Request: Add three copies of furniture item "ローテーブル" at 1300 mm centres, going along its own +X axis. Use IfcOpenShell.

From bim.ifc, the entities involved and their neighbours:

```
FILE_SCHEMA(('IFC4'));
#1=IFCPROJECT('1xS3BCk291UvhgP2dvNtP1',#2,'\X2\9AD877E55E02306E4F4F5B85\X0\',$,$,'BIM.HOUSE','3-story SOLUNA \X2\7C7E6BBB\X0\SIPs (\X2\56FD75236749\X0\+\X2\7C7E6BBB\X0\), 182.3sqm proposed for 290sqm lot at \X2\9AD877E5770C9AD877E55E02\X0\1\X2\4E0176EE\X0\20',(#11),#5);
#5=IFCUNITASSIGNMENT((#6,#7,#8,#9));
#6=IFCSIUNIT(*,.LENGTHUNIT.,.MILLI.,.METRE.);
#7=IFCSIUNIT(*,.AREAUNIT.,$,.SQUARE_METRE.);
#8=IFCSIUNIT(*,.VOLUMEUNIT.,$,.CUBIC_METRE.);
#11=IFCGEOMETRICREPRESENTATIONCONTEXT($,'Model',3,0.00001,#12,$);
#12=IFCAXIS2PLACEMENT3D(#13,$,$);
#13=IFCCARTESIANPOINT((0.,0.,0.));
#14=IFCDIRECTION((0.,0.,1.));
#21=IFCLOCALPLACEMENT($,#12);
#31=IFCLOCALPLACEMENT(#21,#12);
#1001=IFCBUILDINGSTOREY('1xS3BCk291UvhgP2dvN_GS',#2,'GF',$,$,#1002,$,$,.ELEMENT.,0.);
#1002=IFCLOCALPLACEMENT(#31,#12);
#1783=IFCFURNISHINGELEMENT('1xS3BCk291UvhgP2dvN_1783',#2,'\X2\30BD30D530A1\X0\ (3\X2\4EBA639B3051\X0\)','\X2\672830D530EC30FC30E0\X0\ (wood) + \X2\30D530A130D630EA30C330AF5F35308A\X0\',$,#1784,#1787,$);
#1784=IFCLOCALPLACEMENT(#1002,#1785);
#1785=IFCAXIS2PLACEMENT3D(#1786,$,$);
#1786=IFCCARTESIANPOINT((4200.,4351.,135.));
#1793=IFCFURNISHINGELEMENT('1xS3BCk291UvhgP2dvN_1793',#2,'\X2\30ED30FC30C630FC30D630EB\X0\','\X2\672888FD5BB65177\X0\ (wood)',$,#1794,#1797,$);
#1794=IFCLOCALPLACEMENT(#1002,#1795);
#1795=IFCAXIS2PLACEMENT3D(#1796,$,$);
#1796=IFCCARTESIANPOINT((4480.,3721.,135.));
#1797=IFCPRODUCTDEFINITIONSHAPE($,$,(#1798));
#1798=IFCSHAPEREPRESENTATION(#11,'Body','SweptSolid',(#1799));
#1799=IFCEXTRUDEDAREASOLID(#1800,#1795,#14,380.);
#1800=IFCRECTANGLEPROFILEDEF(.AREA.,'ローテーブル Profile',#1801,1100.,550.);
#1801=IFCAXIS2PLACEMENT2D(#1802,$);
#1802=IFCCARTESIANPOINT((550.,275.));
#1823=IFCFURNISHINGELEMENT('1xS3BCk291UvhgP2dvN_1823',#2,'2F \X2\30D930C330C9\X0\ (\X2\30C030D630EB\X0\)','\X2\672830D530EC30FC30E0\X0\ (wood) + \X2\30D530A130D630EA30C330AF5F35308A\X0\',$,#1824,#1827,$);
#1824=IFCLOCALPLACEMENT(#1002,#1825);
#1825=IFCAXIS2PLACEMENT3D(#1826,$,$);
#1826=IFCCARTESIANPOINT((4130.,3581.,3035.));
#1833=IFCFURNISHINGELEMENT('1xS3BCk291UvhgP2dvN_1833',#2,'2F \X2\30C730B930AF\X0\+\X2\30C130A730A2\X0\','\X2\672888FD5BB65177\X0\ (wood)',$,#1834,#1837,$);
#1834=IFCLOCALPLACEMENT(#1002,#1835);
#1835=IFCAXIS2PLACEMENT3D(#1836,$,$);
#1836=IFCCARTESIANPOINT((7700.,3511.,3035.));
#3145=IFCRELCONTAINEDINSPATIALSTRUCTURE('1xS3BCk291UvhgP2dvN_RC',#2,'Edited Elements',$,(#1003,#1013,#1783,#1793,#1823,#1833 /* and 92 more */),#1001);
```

```python
import ifcopenshell
import ifcopenshell.api.geometry
import ifcopenshell.api.root
import ifcopenshell.util.element
import ifcopenshell.util.placement

model = ifcopenshell.open("bim.ifc")


def reuse_history(source, copy):
    """copy_class also copies each property set's owner history, people and application; keep the originals."""
    for rel in copy.IsDefinedBy:
        if rel.is_a("IfcRelDefinesByProperties") and (history := rel.RelatingPropertyDefinition.OwnerHistory):
            rel.RelatingPropertyDefinition.OwnerHistory = source.OwnerHistory
            ifcopenshell.util.element.remove_deep2(model, history)


source = model.by_guid("1xS3BCk291UvhgP2dvN_1793")
base = ifcopenshell.util.placement.get_local_placement(source.ObjectPlacement)
step = base[:3, 0] * 1300.0

for i in range(1, 4):
    copy = ifcopenshell.api.root.copy_class(model, product=source)
    copy.Representation = ifcopenshell.util.element.copy_deep(
        model, source.Representation, exclude=["IfcGeometricRepresentationContext", "IfcRepresentationMap"]
    )
    reuse_history(source, copy)
    matrix = base.copy()
    matrix[:3, 3] += i * step
    print("added at", matrix[:3, 3].round(3) + 0.0)
    ifcopenshell.api.geometry.edit_object_placement(model, product=copy, matrix=matrix, is_si=False)

model.write("bim_edited.ifc")
```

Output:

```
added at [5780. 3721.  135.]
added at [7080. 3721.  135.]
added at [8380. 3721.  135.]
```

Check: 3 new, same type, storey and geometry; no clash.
